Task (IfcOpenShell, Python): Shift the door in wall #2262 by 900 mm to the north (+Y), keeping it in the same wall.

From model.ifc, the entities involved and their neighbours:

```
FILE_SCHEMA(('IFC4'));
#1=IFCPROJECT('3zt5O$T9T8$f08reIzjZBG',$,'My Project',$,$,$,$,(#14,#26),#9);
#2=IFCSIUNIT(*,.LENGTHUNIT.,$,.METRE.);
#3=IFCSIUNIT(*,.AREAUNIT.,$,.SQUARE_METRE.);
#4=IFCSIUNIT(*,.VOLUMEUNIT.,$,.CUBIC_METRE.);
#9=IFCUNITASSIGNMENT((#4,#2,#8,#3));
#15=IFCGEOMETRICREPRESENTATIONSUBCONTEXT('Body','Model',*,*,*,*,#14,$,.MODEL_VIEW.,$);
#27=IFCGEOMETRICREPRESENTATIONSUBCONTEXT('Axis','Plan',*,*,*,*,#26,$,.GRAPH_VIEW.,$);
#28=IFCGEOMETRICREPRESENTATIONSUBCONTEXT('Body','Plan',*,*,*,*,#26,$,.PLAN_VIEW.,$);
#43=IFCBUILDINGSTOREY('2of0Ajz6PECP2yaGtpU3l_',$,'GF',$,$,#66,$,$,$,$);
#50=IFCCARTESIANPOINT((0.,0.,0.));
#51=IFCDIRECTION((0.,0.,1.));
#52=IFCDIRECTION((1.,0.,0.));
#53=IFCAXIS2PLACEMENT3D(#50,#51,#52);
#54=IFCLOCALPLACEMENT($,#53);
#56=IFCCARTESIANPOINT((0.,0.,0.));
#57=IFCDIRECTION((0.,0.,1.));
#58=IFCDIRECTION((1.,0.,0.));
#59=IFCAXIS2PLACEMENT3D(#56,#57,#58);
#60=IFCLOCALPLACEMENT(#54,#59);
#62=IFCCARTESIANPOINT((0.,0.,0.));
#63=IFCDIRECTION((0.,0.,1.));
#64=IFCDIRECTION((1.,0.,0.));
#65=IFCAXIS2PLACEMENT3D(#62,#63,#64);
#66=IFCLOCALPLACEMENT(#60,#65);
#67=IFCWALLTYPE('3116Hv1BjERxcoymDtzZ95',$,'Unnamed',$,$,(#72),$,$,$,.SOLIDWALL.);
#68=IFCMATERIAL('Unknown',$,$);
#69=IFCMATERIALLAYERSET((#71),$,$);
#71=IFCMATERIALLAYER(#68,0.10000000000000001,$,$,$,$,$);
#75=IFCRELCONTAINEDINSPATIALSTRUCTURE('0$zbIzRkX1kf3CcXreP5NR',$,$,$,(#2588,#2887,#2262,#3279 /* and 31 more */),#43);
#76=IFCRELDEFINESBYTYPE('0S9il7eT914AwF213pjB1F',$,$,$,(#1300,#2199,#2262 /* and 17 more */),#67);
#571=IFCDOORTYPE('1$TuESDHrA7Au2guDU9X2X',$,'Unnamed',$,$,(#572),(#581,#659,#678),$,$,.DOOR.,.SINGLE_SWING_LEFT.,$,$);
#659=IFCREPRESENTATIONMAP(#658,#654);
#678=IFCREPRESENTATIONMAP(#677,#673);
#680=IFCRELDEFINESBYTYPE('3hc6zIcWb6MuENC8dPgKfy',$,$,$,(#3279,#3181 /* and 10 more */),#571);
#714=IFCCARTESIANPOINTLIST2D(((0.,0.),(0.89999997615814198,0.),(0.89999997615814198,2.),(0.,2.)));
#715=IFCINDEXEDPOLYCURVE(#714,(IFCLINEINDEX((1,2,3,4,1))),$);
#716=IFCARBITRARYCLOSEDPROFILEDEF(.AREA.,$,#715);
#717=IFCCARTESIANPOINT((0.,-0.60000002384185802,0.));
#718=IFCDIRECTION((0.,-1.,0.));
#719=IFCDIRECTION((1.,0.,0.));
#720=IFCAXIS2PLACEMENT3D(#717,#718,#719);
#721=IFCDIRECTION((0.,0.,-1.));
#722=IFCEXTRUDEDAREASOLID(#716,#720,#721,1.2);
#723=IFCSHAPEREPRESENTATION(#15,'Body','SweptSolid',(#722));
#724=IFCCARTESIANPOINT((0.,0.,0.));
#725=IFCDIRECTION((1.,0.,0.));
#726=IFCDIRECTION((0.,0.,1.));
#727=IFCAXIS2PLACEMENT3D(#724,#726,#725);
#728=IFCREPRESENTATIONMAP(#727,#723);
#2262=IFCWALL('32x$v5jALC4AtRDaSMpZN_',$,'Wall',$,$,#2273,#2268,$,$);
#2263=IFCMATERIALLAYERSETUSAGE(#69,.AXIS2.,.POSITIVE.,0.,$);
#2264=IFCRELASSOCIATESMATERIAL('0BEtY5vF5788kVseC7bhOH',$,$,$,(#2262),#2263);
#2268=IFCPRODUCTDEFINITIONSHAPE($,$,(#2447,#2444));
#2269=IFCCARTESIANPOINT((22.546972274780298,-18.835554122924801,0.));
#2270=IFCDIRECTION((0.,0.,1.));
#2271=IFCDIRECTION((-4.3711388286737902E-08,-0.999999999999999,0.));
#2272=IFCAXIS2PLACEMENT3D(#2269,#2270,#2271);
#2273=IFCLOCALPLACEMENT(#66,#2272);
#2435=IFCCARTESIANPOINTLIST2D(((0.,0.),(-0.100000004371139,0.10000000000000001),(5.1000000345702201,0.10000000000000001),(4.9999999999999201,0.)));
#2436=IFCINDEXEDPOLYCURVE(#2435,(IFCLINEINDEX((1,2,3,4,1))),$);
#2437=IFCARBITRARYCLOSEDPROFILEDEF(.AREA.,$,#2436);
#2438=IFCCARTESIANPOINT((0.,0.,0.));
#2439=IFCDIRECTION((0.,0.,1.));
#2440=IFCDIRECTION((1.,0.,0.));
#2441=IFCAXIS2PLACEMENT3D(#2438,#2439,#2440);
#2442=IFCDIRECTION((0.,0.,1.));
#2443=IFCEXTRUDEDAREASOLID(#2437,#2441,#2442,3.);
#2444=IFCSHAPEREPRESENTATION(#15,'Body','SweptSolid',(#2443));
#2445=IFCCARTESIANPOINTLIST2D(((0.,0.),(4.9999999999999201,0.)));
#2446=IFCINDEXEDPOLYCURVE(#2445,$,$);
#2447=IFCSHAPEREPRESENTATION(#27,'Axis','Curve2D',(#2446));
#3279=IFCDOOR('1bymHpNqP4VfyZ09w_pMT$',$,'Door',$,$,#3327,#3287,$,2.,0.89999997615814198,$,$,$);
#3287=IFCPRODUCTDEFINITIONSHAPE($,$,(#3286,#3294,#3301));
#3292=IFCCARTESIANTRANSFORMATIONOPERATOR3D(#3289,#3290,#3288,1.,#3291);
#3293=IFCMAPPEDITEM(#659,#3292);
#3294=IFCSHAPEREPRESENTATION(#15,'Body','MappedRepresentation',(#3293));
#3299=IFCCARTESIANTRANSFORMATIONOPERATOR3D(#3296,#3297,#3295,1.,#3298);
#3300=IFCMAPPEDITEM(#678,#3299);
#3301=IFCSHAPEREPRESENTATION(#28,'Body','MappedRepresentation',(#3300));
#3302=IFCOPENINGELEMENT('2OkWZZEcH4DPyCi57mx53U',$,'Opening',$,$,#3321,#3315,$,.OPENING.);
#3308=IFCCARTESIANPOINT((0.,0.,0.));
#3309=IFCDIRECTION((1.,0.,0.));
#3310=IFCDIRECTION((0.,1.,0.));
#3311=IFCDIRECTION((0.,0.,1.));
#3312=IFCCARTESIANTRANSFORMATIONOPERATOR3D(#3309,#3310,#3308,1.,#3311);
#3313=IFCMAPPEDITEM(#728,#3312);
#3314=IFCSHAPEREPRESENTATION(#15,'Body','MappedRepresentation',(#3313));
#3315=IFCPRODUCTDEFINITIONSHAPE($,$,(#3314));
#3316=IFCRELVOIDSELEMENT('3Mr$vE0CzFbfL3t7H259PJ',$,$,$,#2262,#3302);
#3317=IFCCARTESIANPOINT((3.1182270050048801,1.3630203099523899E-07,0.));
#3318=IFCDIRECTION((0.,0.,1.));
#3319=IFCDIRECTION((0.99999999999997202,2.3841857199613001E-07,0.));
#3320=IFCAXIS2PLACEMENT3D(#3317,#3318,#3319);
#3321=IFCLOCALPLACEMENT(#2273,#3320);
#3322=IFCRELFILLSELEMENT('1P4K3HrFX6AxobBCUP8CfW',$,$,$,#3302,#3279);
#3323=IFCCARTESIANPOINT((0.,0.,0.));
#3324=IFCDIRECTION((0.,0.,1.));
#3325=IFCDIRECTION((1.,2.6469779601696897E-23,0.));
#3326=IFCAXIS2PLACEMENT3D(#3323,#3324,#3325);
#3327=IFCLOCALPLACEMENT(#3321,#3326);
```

```python
import ifcopenshell
import ifcopenshell.api.geometry
import ifcopenshell.util.placement
import ifcopenshell.util.unit

model = ifcopenshell.open("model.ifc")
unit_scale = ifcopenshell.util.unit.calculate_unit_scale(model)

door = model.by_guid("1bymHpNqP4VfyZ09w_pMT$")
opening = door.FillsVoids[0].RelatingOpeningElement
wall = opening.VoidsElements[0].RelatingBuildingElement

wall_matrix = ifcopenshell.util.placement.get_local_placement(wall.ObjectPlacement)
shift = wall_matrix[:3, 0] * -0.9 / unit_scale
before = ifcopenshell.util.placement.get_local_placement(door.ObjectPlacement)[:3, 3].copy()

# The door is placed relative to its opening, so it follows when the opening moves.
matrix = ifcopenshell.util.placement.get_local_placement(opening.ObjectPlacement)
matrix[:3, 3] += shift
ifcopenshell.api.geometry.edit_object_placement(
    model, product=opening, matrix=matrix, is_si=False, should_transform_children=True
)

after = ifcopenshell.util.placement.get_local_placement(door.ObjectPlacement)[:3, 3]
print("door moved by", (after - before).round(3) + 0.0)

model.write("model_rev.ifc")
```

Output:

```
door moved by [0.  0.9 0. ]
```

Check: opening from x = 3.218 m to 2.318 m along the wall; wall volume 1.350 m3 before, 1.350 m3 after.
